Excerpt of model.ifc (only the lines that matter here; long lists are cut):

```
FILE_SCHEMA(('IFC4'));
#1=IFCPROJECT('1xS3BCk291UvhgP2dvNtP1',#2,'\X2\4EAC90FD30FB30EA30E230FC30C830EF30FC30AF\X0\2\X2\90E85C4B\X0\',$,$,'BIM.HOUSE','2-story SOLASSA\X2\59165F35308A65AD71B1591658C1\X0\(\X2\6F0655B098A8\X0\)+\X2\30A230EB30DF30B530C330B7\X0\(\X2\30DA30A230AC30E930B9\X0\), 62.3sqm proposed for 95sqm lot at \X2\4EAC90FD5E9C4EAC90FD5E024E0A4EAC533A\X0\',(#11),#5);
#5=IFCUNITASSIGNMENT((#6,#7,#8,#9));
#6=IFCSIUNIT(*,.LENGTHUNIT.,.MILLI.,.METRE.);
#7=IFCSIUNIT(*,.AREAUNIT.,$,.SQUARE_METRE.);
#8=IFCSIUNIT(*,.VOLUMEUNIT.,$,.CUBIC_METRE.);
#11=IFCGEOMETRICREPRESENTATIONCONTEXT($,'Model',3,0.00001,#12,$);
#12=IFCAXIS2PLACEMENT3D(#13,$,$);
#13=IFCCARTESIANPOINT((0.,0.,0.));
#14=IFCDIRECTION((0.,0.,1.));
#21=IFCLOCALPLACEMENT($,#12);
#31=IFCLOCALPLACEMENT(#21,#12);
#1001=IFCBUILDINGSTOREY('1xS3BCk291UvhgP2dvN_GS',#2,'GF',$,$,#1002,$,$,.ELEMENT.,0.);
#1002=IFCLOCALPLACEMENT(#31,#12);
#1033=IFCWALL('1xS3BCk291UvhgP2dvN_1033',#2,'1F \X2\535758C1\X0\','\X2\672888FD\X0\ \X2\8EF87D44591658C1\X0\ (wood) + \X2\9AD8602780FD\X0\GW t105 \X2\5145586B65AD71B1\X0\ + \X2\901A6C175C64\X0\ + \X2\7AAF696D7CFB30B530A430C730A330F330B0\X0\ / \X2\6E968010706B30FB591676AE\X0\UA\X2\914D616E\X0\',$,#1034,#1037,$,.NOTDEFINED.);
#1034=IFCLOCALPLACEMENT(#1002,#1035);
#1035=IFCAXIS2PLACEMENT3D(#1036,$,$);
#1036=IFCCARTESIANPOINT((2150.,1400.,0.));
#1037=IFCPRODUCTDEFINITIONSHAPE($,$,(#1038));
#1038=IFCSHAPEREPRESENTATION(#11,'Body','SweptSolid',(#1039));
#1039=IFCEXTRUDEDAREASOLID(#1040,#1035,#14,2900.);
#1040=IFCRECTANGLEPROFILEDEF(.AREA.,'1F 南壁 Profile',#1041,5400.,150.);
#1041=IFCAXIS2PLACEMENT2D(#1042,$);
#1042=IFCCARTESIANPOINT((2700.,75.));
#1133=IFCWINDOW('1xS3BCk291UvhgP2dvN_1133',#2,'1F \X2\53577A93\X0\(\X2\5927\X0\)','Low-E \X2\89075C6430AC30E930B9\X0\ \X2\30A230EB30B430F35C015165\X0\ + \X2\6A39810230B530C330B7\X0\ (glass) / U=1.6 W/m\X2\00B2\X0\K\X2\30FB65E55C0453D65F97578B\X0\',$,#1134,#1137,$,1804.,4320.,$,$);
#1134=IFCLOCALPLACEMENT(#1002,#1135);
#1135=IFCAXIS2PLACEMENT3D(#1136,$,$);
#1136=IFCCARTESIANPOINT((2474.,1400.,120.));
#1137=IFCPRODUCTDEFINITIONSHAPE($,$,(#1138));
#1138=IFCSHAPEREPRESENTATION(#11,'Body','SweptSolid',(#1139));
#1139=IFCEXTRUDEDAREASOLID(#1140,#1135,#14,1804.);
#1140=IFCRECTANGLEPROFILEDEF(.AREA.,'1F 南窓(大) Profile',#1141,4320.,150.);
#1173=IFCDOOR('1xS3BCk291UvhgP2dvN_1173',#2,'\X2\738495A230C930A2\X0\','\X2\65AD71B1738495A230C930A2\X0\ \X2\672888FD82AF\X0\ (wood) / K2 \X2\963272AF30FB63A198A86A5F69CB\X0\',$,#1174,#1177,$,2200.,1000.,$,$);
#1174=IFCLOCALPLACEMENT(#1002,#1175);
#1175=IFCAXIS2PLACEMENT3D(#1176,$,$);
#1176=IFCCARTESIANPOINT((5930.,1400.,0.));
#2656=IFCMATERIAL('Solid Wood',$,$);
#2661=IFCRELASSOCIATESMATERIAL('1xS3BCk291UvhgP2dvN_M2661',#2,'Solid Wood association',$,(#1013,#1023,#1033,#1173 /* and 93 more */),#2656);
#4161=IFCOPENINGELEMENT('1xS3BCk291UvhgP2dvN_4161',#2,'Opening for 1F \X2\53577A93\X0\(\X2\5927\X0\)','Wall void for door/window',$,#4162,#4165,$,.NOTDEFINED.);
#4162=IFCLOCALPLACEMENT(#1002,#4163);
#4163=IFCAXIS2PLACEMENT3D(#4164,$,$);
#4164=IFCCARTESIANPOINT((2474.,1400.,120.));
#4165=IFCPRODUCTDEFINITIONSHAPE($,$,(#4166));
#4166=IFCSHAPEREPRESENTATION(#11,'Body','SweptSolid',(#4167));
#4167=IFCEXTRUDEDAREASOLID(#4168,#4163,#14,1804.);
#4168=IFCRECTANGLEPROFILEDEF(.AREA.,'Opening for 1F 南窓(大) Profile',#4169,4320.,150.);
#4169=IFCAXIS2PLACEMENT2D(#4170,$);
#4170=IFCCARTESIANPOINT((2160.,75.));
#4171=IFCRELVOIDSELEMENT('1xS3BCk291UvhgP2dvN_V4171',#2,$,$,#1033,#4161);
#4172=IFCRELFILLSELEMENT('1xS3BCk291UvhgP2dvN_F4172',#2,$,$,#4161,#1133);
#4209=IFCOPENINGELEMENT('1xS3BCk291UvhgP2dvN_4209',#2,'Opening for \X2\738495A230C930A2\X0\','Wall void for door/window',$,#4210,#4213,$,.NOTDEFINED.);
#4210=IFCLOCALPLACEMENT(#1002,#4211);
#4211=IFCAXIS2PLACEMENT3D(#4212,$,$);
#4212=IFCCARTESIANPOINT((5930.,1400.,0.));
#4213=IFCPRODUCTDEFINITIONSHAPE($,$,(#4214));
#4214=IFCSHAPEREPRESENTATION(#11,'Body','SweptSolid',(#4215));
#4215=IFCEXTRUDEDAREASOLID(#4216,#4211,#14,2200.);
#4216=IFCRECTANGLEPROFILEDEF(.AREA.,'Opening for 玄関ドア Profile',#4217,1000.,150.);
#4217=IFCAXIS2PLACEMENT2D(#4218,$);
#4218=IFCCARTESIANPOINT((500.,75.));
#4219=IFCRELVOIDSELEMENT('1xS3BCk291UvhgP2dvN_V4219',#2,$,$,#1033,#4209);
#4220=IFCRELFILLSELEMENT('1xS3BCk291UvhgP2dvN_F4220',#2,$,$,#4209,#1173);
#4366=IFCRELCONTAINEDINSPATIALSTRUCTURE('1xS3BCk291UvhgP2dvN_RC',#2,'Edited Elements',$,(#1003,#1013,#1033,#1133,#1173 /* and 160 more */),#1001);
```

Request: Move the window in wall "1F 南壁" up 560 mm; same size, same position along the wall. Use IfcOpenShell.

```python
import numpy as np
import ifcopenshell
import ifcopenshell.api.geometry
import ifcopenshell.util.placement
import ifcopenshell.util.unit

model = ifcopenshell.open("model.ifc")
unit_scale = ifcopenshell.util.unit.calculate_unit_scale(model)

window = model.by_id(1133)
opening = window.FillsVoids[0].RelatingOpeningElement
dz = 0.56 / unit_scale

shift = np.array([0.0, 0.0, dz])
# The window is not placed relative to its opening, so move both.
for product in (opening, window):
    matrix = ifcopenshell.util.placement.get_local_placement(product.ObjectPlacement)
    matrix[:3, 3] += shift
    ifcopenshell.api.geometry.edit_object_placement(model, product=product, matrix=matrix, is_si=False)

print(f"moved by {dz * unit_scale:+.3f} m")

model.write("model_rev.ifc")
```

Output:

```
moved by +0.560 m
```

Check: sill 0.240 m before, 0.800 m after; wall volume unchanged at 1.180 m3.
